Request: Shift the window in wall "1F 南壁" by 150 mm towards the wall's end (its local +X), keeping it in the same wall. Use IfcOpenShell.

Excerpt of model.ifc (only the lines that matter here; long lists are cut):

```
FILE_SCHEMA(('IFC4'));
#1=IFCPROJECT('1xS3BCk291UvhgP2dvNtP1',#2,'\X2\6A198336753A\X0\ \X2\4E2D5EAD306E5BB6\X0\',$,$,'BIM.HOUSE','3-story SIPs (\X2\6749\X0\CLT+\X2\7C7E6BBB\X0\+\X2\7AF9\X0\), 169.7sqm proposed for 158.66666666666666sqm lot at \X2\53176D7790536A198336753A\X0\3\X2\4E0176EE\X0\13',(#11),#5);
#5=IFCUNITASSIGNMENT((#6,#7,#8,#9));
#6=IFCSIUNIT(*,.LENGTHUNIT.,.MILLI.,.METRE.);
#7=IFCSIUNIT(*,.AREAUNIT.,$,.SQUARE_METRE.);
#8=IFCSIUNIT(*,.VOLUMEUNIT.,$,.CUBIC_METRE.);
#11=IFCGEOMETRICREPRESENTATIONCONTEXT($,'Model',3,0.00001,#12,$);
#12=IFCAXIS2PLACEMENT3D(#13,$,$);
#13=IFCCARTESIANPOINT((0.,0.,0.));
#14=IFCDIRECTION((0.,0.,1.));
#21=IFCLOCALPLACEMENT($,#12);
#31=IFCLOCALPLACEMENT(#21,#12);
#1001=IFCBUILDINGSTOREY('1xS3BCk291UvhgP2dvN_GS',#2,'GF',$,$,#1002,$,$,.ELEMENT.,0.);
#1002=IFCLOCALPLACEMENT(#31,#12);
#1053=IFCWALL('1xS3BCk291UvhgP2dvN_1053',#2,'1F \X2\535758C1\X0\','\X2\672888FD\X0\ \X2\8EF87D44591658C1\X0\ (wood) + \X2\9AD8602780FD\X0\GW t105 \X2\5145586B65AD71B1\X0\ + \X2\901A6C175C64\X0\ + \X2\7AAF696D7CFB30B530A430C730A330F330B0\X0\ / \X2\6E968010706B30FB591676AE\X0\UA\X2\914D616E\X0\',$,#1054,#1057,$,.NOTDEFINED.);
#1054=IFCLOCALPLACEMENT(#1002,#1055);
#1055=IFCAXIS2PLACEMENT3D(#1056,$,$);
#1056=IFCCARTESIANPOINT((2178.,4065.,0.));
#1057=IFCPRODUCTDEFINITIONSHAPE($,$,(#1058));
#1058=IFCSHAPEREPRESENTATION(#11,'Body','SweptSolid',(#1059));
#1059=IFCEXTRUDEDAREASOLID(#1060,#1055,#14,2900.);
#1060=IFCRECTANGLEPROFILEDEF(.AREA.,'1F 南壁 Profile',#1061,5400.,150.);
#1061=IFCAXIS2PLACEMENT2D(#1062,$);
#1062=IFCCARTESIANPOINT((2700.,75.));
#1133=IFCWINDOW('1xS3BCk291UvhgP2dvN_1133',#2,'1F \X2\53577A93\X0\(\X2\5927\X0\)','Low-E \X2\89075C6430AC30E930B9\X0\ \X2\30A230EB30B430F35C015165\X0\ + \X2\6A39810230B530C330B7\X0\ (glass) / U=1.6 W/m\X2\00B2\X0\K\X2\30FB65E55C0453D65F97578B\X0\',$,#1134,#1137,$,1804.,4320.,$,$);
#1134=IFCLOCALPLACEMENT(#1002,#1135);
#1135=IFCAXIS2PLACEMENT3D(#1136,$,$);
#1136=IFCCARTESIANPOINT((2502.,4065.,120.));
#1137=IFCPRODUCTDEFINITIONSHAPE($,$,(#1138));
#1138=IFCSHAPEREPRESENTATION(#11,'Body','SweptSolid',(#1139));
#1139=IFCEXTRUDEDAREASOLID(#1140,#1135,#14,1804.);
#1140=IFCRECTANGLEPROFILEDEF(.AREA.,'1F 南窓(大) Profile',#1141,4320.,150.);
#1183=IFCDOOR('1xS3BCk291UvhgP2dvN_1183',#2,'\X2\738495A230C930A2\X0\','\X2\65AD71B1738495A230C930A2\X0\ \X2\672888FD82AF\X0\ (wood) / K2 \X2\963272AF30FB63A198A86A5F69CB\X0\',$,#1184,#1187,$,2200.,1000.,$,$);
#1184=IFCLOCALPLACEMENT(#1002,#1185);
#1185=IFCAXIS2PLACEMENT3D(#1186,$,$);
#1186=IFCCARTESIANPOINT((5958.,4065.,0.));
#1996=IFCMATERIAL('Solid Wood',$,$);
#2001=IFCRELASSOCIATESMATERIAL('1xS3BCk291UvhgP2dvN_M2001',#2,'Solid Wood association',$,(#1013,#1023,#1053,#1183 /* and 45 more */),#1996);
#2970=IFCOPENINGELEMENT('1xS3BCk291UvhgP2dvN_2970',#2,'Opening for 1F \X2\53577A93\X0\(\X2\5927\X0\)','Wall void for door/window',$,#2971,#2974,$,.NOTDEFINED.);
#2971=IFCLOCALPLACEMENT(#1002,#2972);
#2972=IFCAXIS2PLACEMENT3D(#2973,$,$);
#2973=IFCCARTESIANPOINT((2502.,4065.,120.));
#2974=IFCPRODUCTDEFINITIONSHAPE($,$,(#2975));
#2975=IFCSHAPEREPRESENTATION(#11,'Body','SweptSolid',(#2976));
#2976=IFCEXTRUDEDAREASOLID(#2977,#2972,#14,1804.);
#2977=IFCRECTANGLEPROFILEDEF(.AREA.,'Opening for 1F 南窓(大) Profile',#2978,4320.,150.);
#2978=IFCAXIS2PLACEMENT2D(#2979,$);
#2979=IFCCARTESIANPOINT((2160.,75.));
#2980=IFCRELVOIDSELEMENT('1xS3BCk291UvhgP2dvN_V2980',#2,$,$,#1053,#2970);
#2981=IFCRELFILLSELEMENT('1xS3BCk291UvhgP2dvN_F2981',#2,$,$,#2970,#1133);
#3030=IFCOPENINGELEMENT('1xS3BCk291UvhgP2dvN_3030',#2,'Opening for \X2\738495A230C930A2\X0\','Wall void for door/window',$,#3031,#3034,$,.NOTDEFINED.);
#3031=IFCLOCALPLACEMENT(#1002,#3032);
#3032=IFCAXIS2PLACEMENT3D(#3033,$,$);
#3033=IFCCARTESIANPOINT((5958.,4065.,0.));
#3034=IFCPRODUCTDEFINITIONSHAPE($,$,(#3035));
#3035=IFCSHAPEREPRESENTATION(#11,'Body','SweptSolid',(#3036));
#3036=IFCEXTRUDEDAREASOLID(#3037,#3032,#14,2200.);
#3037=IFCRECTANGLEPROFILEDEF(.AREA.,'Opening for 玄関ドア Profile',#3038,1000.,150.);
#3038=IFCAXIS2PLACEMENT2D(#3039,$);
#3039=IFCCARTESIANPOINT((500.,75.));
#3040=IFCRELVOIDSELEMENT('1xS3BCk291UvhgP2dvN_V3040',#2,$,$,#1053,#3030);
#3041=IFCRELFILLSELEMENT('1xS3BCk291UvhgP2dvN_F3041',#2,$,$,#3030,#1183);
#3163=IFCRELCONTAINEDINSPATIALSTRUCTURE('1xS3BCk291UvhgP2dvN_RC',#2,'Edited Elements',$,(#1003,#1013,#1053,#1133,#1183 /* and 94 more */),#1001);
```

```python
import ifcopenshell
import ifcopenshell.api.geometry
import ifcopenshell.util.placement
import ifcopenshell.util.unit

model = ifcopenshell.open("model.ifc")
unit_scale = ifcopenshell.util.unit.calculate_unit_scale(model)

window = model.by_guid("1xS3BCk291UvhgP2dvN_1133")
opening = window.FillsVoids[0].RelatingOpeningElement
wall = opening.VoidsElements[0].RelatingBuildingElement

wall_matrix = ifcopenshell.util.placement.get_local_placement(wall.ObjectPlacement)
shift = wall_matrix[:3, 0] * 0.15 / unit_scale
before = ifcopenshell.util.placement.get_local_placement(window.ObjectPlacement)[:3, 3].copy()

# The window is not placed relative to its opening, so move both.
for product in (opening, window):
    matrix = ifcopenshell.util.placement.get_local_placement(product.ObjectPlacement)
    matrix[:3, 3] += shift
    ifcopenshell.api.geometry.edit_object_placement(model, product=product, matrix=matrix, is_si=False)

after = ifcopenshell.util.placement.get_local_placement(window.ObjectPlacement)[:3, 3]
print("window moved by", (after - before).round(3) + 0.0)

model.write("model_v2.ifc")
```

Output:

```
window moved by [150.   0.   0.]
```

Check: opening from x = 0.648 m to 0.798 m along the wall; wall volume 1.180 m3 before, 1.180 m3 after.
